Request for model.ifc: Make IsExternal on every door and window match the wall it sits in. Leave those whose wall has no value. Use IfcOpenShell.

First a look at what the model holds.

```python
import ifcopenshell
import ifcopenshell.util.element

model = ifcopenshell.open("model.ifc")
print(model.schema)
seen = {}
for e in model.by_type("IfcDoor") + model.by_type("IfcWindow"):
    if not e.FillsVoids:
        continue
    host = e.FillsVoids[0].RelatingOpeningElement.VoidsElements[0].RelatingBuildingElement
    own = ifcopenshell.util.element.get_pset(e, f"Pset_{e.is_a()[3:].removesuffix('StandardCase')}Common", "IsExternal")
    wall = ifcopenshell.util.element.get_pset(host, "Pset_WallCommon", "IsExternal")
    seen[e.is_a(), own, wall] = seen.get((e.is_a(), own, wall), 0) + 1
for (cls, own, wall), count in sorted(seen.items(), key=str):
    print(count, cls, "IsExternal:", own, "| host wall:", wall)
```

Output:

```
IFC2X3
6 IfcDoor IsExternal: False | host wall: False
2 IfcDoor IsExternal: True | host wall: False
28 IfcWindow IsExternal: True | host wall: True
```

```python
import ifcopenshell
import ifcopenshell.api.pset
import ifcopenshell.util.element

model = ifcopenshell.open("model.ifc")

count = 0
for ifc_class, pset_name in (("IfcDoor", "Pset_DoorCommon"), ("IfcWindow", "Pset_WindowCommon")):
    for e in model.by_type(ifc_class):
        if not e.FillsVoids:
            continue
        host = e.FillsVoids[0].RelatingOpeningElement.VoidsElements[0].RelatingBuildingElement
        external = ifcopenshell.util.element.get_pset(host, "Pset_WallCommon", "IsExternal")
        if external is None or ifcopenshell.util.element.get_pset(e, pset_name, "IsExternal") == external:
            continue
        pset = ifcopenshell.api.pset.add_pset(model, product=e, name=pset_name)
        ifcopenshell.api.pset.edit_pset(model, pset=pset, properties={"IsExternal": external})
        count += 1

print(count, "updated")

model.write("model-out.ifc")
```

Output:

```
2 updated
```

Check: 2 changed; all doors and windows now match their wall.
